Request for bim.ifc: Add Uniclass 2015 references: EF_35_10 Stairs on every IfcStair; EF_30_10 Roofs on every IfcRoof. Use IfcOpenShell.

First a look at what the model holds.

```python
import ifcopenshell

model = ifcopenshell.open("bim.ifc")
print(model.schema)
print("classifications:", [c.Name for c in model.by_type("IfcClassification")])
for ifc_class in ("IfcDoor", "IfcRoof", "IfcStair", "IfcWall", "IfcWindow"):
    print(ifc_class, len(model.by_type(ifc_class)))
```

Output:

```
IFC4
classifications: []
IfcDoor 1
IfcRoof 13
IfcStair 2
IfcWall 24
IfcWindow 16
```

```python
import ifcopenshell
import ifcopenshell.api.classification

model = ifcopenshell.open("bim.ifc")

system = ifcopenshell.api.classification.add_classification(model, classification="Uniclass 2015")

codes = {
    "IfcStair": ("EF_35_10", "Stairs"),
    "IfcRoof": ("EF_30_10", "Roofs"),
}
for ifc_class, (code, name) in codes.items():
    products = model.by_type(ifc_class)
    ifcopenshell.api.classification.add_reference(
        model, products=products, classification=system, identification=code, name=name
    )
    print(code, len(products))

model.write("bim_v2.ifc")
```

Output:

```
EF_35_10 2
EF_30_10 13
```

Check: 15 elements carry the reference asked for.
